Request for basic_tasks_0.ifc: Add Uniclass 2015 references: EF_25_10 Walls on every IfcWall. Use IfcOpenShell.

First a look at what the model holds.

```python
import ifcopenshell

model = ifcopenshell.open("basic_tasks_0.ifc")
print(model.schema)
print("classifications:", [c.Name for c in model.by_type("IfcClassification")])
for ifc_class in ("IfcDoor", "IfcRoof", "IfcStair", "IfcWall", "IfcWindow"):
    print(ifc_class, len(model.by_type(ifc_class)))
```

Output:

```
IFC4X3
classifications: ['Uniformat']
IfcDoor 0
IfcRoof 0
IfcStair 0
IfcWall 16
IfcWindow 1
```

```python
import ifcopenshell
import ifcopenshell.api.classification

model = ifcopenshell.open("basic_tasks_0.ifc")

system = ifcopenshell.api.classification.add_classification(model, classification="Uniclass 2015")

codes = {
    "IfcWall": ("EF_25_10", "Walls"),
}
for ifc_class, (code, name) in codes.items():
    products = model.by_type(ifc_class)
    ifcopenshell.api.classification.add_reference(
        model, products=products, classification=system, identification=code, name=name
    )
    print(code, len(products))

model.write("basic_tasks_0_rev.ifc")
```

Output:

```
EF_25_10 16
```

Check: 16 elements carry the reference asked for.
